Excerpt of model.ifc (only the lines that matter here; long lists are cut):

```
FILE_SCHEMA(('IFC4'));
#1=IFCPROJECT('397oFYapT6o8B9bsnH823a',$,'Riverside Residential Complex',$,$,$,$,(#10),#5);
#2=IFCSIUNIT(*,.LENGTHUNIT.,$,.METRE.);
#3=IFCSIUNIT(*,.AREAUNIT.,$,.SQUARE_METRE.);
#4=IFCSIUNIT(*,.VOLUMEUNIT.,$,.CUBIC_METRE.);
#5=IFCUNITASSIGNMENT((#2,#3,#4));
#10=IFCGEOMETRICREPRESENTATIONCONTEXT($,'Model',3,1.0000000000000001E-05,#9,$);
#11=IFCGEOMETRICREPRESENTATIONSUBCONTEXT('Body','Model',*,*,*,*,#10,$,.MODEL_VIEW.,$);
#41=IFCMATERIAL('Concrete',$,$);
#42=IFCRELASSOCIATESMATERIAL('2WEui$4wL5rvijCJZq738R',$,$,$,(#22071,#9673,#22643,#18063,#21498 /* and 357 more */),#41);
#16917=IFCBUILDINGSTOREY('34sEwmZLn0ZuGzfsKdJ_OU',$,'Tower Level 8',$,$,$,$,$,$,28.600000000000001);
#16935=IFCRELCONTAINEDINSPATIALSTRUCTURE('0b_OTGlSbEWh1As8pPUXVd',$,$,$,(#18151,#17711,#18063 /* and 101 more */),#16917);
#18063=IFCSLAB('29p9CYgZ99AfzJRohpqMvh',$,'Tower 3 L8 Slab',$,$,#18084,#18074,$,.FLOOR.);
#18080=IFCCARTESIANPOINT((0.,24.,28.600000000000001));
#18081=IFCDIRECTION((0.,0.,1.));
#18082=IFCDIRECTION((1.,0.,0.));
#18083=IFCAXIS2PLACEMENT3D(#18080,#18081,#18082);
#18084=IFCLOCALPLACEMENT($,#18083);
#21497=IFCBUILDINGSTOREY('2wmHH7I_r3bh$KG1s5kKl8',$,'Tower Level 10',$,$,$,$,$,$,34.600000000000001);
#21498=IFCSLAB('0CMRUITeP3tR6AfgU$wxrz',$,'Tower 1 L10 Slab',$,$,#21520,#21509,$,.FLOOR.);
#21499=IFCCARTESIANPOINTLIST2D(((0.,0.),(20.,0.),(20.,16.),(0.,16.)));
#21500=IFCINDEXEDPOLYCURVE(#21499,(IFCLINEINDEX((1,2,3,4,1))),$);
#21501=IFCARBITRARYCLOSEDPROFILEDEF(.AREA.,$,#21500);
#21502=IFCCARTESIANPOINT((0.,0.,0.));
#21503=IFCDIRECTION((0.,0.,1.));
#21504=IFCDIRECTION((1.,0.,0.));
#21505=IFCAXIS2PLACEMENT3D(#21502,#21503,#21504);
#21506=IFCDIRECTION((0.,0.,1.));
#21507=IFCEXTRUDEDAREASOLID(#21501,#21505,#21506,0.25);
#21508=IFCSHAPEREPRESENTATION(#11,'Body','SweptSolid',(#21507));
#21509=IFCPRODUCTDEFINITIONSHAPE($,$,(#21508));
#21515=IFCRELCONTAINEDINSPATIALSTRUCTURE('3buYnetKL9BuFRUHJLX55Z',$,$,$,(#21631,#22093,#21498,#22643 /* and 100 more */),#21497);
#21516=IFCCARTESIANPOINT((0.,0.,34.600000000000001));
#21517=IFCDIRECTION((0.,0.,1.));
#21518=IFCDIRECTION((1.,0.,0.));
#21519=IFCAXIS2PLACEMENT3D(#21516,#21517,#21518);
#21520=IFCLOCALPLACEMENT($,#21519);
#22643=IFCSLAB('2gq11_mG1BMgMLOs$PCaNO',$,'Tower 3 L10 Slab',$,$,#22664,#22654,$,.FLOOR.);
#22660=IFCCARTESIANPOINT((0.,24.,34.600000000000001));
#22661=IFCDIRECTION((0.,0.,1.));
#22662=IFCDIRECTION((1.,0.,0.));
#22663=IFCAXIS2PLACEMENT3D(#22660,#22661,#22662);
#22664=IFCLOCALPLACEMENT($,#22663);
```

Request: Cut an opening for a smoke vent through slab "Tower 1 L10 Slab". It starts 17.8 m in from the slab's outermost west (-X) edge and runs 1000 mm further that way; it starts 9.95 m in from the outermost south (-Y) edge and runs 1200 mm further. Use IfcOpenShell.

```python
import numpy as np
import ifcopenshell
import ifcopenshell.api.feature
import ifcopenshell.api.geometry
import ifcopenshell.api.root
import ifcopenshell.geom
import ifcopenshell.util.placement
import ifcopenshell.util.representation
import ifcopenshell.util.shape
import ifcopenshell.util.unit

model = ifcopenshell.open("model.ifc")
unit_scale = ifcopenshell.util.unit.calculate_unit_scale(model)
settings = ifcopenshell.geom.settings()


def volume(element):
    """Net volume in cubic metres, openings subtracted."""
    shape = ifcopenshell.geom.create_shape(settings, element)
    return ifcopenshell.util.shape.get_volume(shape.geometry)


slab = model.by_guid("0CMRUITeP3tR6AfgU$wxrz")
before = volume(slab)

# Extent in the slab's own axes, in metres. The edges named are its -X and -Y sides.
slab_shape = ifcopenshell.geom.create_shape(settings, slab)
vertices = ifcopenshell.util.shape.get_vertices(slab_shape.geometry)
x_min, y_min, bottom = vertices.min(axis=0)
top = vertices[:, 2].max()

opening = ifcopenshell.api.root.create_entity(model, ifc_class="IfcOpeningElement", name="Smoke vent opening", predefined_type="OPENING")
context = ifcopenshell.util.representation.get_context(model, "Model", "Body", "MODEL_VIEW")
width, depth = 1, 1.2
outline = [(0.0, 0.0), (width, 0.0), (width, depth), (0.0, depth), (0.0, 0.0)]
# Overshoot both faces by 50 mm so the cut is clean.
shape = ifcopenshell.api.geometry.add_slab_representation(
    model, context=context, depth=top - bottom + 0.1, polyline=outline
)
ifcopenshell.api.geometry.assign_representation(model, product=opening, representation=shape)

matrix = ifcopenshell.util.placement.get_local_placement(slab.ObjectPlacement)
matrix[:, 3] = matrix @ np.append(np.array([x_min + 17.8, y_min + 9.95, bottom - 0.05]) / unit_scale, 1.0)
ifcopenshell.api.geometry.edit_object_placement(model, product=opening, matrix=matrix, is_si=False)
ifcopenshell.api.feature.add_feature(model, feature=opening, element=slab)

after = volume(slab)

print(f"slab volume {before:.3f} -> {after:.3f} m3")

model.write("model_rev.ifc")
```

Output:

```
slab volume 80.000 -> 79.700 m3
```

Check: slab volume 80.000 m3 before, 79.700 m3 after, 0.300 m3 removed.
